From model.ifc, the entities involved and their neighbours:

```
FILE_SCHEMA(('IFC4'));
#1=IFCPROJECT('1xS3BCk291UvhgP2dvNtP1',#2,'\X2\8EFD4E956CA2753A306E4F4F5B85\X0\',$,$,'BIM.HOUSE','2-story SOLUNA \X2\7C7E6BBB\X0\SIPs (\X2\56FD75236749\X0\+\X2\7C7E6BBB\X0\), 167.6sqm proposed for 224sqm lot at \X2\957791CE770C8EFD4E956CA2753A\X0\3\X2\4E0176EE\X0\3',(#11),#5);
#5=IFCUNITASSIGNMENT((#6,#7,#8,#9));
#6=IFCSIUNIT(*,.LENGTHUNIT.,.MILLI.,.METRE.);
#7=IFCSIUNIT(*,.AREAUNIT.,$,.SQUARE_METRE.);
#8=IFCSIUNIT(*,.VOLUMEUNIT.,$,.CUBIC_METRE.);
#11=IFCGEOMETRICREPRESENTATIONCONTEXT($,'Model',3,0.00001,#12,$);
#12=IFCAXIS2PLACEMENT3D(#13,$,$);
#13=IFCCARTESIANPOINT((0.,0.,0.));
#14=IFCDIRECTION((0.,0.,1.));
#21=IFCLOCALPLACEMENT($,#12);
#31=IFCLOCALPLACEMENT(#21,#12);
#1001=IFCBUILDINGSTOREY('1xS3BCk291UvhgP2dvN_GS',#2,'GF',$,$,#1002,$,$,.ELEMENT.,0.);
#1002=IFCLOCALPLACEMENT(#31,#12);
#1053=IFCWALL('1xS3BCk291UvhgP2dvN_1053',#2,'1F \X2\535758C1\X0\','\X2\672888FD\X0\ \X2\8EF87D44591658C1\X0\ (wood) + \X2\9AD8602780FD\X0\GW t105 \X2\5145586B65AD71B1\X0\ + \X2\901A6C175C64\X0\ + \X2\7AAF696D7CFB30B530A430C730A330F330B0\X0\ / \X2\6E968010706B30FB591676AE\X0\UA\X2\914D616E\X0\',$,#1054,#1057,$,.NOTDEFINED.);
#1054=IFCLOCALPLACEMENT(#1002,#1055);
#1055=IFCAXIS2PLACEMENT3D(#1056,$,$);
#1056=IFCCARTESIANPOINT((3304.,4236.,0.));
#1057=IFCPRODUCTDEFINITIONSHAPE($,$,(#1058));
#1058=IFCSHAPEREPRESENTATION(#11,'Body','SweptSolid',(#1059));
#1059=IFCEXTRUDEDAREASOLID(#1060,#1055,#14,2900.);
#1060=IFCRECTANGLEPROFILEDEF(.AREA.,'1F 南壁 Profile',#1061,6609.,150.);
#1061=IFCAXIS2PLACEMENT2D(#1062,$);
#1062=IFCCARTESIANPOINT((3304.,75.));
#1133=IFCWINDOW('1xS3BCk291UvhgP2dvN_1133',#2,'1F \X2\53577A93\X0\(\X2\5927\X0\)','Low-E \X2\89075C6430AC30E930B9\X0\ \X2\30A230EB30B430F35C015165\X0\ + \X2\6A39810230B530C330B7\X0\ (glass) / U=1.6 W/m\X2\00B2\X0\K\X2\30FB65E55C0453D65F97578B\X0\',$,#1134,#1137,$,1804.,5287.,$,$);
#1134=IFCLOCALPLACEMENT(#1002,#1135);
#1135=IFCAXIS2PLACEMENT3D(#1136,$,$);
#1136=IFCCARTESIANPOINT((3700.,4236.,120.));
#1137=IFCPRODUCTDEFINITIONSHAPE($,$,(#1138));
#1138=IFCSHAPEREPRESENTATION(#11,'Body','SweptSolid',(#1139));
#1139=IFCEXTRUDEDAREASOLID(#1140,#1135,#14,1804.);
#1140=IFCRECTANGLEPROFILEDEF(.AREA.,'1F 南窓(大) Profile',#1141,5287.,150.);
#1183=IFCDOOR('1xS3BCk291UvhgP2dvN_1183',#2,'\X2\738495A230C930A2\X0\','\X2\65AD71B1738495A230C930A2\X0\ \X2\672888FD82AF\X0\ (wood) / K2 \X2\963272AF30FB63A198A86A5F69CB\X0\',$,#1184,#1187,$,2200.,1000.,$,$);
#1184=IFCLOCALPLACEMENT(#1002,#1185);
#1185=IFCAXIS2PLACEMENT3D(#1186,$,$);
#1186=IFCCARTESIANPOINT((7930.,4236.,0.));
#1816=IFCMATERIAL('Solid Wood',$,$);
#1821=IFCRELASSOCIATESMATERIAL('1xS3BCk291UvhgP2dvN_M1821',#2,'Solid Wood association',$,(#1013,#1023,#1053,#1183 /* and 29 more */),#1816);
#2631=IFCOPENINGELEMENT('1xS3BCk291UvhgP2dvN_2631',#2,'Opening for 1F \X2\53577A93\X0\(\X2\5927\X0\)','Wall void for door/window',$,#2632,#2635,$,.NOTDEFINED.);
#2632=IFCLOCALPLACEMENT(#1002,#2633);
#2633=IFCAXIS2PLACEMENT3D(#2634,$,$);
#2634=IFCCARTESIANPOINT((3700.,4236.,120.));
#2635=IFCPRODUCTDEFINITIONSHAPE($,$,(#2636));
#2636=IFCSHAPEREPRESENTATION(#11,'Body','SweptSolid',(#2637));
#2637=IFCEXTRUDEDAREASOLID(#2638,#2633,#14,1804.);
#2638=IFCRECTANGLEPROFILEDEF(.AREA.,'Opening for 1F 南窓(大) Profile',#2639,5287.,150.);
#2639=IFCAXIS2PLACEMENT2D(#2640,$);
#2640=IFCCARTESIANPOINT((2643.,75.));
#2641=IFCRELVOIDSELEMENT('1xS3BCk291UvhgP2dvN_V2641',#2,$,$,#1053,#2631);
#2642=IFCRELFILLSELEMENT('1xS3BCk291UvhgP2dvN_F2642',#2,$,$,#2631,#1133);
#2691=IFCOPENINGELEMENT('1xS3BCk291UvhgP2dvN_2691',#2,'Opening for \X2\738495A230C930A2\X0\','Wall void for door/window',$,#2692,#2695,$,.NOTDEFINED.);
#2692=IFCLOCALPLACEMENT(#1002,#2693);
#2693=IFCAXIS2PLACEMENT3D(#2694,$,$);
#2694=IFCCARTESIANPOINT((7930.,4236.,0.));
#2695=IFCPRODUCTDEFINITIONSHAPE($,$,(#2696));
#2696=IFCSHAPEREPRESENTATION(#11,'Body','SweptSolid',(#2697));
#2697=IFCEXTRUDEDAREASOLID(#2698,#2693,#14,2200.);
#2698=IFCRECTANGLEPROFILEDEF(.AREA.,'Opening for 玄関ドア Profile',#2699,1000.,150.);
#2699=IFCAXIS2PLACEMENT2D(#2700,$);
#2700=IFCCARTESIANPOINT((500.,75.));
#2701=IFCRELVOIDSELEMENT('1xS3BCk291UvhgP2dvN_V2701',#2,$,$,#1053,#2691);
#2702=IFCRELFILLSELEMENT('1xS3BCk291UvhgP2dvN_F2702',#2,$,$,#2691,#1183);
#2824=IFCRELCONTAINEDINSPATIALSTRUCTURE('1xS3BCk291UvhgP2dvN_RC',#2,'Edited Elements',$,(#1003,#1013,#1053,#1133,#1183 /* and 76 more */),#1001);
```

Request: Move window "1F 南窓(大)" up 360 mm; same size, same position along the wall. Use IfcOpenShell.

```python
import numpy as np
import ifcopenshell
import ifcopenshell.api.geometry
import ifcopenshell.util.placement
import ifcopenshell.util.unit

model = ifcopenshell.open("model.ifc")
unit_scale = ifcopenshell.util.unit.calculate_unit_scale(model)

window = model.by_guid("1xS3BCk291UvhgP2dvN_1133")
opening = window.FillsVoids[0].RelatingOpeningElement
dz = 360.0

shift = np.array([0.0, 0.0, dz])
# The window is not placed relative to its opening, so move both.
for product in (opening, window):
    matrix = ifcopenshell.util.placement.get_local_placement(product.ObjectPlacement)
    matrix[:3, 3] += shift
    ifcopenshell.api.geometry.edit_object_placement(model, product=product, matrix=matrix, is_si=False)

print(f"moved by {dz * unit_scale:+.3f} m")

model.write("model_rev.ifc")
```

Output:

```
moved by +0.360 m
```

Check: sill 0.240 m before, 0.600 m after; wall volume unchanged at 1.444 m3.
